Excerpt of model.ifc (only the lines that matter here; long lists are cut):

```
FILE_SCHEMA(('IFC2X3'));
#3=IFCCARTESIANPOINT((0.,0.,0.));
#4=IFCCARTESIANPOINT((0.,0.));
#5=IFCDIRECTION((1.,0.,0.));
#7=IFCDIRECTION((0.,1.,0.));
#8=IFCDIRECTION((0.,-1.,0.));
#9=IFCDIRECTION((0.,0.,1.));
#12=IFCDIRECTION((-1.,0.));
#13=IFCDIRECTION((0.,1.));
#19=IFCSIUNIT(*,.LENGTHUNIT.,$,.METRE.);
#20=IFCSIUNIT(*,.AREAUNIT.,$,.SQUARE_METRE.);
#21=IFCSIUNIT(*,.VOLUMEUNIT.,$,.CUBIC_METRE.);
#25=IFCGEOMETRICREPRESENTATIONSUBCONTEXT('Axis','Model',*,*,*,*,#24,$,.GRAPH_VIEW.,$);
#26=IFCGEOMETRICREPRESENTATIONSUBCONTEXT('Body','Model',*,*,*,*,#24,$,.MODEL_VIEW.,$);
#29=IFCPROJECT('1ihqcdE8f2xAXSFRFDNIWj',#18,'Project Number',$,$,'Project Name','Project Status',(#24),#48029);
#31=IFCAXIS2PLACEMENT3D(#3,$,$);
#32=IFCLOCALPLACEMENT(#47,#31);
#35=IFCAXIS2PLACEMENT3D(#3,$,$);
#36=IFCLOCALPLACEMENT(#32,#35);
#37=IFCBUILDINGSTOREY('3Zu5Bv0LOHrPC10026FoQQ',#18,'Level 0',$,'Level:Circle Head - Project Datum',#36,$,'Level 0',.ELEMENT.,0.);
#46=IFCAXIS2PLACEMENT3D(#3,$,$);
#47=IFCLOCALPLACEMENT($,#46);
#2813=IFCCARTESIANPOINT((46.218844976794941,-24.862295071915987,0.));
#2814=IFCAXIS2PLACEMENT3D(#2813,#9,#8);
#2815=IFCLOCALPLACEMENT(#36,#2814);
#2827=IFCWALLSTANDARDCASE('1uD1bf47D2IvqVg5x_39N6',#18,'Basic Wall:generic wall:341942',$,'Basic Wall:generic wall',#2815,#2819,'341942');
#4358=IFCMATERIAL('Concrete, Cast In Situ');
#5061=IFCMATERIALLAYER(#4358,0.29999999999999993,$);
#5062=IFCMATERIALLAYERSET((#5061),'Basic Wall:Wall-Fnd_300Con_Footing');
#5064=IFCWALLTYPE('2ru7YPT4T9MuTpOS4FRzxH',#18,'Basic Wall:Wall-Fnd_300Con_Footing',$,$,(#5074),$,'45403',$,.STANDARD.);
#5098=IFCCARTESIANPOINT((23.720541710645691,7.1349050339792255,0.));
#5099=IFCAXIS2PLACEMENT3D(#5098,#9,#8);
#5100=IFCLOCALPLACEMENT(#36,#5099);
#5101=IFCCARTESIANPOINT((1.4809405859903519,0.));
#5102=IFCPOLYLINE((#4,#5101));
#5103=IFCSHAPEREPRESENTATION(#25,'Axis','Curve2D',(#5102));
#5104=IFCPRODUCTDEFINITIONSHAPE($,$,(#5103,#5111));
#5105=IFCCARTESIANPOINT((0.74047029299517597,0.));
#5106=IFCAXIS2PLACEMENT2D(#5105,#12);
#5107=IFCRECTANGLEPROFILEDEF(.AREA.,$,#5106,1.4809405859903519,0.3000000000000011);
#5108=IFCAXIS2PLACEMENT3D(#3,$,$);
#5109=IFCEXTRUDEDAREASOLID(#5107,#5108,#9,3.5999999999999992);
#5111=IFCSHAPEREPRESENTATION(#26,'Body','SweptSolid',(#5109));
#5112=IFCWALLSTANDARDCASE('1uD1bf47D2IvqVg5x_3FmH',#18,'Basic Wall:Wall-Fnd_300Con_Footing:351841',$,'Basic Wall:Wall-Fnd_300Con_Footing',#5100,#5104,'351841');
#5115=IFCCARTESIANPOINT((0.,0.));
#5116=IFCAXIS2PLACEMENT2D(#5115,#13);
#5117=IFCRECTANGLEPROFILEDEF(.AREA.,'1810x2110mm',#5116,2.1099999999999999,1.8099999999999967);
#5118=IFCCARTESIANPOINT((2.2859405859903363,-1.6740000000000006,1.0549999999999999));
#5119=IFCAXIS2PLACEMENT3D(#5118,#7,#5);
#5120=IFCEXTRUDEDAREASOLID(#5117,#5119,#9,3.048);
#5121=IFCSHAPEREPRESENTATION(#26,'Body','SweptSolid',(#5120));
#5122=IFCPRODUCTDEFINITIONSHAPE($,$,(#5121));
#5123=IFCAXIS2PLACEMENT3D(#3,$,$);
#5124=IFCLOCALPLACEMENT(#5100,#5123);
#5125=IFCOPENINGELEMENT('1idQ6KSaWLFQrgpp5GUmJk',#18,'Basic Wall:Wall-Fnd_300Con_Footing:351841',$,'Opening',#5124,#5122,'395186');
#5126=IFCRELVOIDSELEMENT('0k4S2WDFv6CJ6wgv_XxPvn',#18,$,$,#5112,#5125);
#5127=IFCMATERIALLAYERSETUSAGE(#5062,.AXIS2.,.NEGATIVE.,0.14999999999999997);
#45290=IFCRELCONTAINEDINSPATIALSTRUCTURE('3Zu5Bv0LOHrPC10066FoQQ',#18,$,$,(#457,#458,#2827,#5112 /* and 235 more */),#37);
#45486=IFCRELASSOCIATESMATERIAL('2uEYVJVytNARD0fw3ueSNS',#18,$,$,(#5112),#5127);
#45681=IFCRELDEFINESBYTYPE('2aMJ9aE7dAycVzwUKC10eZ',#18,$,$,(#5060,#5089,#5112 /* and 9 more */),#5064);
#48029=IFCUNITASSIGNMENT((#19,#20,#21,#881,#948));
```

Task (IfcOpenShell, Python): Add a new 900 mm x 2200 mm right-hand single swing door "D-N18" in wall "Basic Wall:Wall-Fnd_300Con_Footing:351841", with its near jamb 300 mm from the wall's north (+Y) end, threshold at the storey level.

```python
import numpy as np
import ifcopenshell
import ifcopenshell.api.feature
import ifcopenshell.api.geometry
import ifcopenshell.api.root
import ifcopenshell.api.spatial
import ifcopenshell.api.type
import ifcopenshell.geom
import ifcopenshell.util.element
import ifcopenshell.util.placement
import ifcopenshell.util.representation
import ifcopenshell.util.shape
import ifcopenshell.util.unit

model = ifcopenshell.open("model.ifc")
unit_scale = ifcopenshell.util.unit.calculate_unit_scale(model)
settings = ifcopenshell.geom.settings()


def volume(element):
    """Net volume in cubic metres, openings subtracted."""
    shape = ifcopenshell.geom.create_shape(settings, element)
    return ifcopenshell.util.shape.get_volume(shape.geometry)


wall = model.by_guid("1uD1bf47D2IvqVg5x_3FmH")
storey = ifcopenshell.util.element.get_container(wall, ifc_class="IfcBuildingStorey")
context = ifcopenshell.util.representation.get_context(model, "Model", "Body", "MODEL_VIEW")
before = volume(wall)

width, height, from_end, sill = 0.9, 2.2, 0.3, 0.0  # metres

# The wall runs along its own X axis, and the end named is its -X end.
wall_shape = ifcopenshell.geom.create_shape(settings, wall)
x, y, z = ifcopenshell.util.shape.get_vertices(wall_shape.geometry).T
start = x.min() + from_end
face, thickness = float(y.min()), float(y.max() - y.min())
wall_matrix = ifcopenshell.util.placement.get_local_placement(wall.ObjectPlacement)
level = ifcopenshell.util.placement.get_local_placement(storey.ObjectPlacement)[2, 3]


def in_wall(x, y):
    """Placement at x, y metres in the wall's axes, at sill height."""
    matrix = wall_matrix.copy()
    matrix[:, 3] = wall_matrix @ np.array([x / unit_scale, y / unit_scale, 0.0, 1.0])
    matrix[2, 3] = level + sill / unit_scale
    return matrix


# Opening: a box that overshoots both wall faces by 50 mm.
opening = ifcopenshell.api.root.create_entity(model, ifc_class="IfcOpeningElement")
box = ifcopenshell.api.geometry.add_wall_representation(
    model, context=context, length=width, height=height, thickness=thickness + 0.1
)
ifcopenshell.api.geometry.assign_representation(model, product=opening, representation=box)
ifcopenshell.api.geometry.edit_object_placement(model, product=opening, matrix=in_wall(start, face - 0.05), is_si=False)
ifcopenshell.api.feature.add_feature(model, feature=opening, element=wall)

door = ifcopenshell.api.root.create_entity(model, ifc_class="IfcDoor", name="D-N18")
door.OverallWidth, door.OverallHeight = width / unit_scale, height / unit_scale
body = ifcopenshell.api.geometry.add_door_representation(
    model,
    context=context,
    overall_width=door.OverallWidth,
    overall_height=door.OverallHeight,
    operation_type="SINGLE_SWING_RIGHT",
    lining_properties={"LiningDepth": thickness / unit_scale, "ThresholdDepth": thickness / unit_scale},
)
ifcopenshell.api.geometry.assign_representation(model, product=door, representation=body)
ifcopenshell.api.spatial.assign_container(model, products=[door], relating_structure=storey)
fills = ifcopenshell.api.feature.add_filling(model, opening=opening, element=door)
fills.OwnerHistory = door.OwnerHistory  # required in IFC2X3

# IFC2X3 keeps the operation on the door style.
style = ifcopenshell.api.root.create_entity(model, ifc_class="IfcDoorStyle", name="D-N18")
style.OperationType, style.ConstructionType = "SINGLE_SWING_RIGHT", "NOTDEFINED"
style.ParameterTakesPrecedence = style.Sizeable = False
ifcopenshell.api.type.assign_type(model, related_objects=[door], relating_type=style)

# The lining spans the wall, so the door starts at the wall face.
ifcopenshell.api.geometry.edit_object_placement(model, product=door, matrix=in_wall(start, face), is_si=False)

after = volume(wall)

print(f"wall volume {before:.3f} -> {after:.3f} m3")

model.write("model_rev.ifc")
```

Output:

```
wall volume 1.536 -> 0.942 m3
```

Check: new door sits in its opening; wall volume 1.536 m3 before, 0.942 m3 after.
